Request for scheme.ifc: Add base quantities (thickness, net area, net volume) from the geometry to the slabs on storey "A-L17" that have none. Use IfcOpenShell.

First a look at what the model holds.

```python
import ifcopenshell
import ifcopenshell.util.element
import ifcopenshell.util.unit

model = ifcopenshell.open("scheme.ifc")
print(model.schema)
for unit_type in ("LENGTHUNIT", "AREAUNIT", "VOLUMEUNIT"):
    print(unit_type, ifcopenshell.util.unit.calculate_unit_scale(model, unit_type))
storey = next(s for s in model.by_type("IfcBuildingStorey") if s.Name == "A-L17")
slabs = [e for e in ifcopenshell.util.element.get_decomposition(storey) if e.is_a("IfcSlab")]
for e in sorted(slabs, key=lambda e: e.id()):
    print(e.id(), e.is_a(), e.Name, list(ifcopenshell.util.element.get_psets(e, qtos_only=True)), sep=" | ")
```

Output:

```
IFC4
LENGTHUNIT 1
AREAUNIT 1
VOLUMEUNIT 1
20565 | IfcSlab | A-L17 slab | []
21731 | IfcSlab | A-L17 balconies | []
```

```python
import ifcopenshell
import ifcopenshell.api.pset
import ifcopenshell.geom
import ifcopenshell.util.element
import ifcopenshell.util.shape
import ifcopenshell.util.unit

model = ifcopenshell.open("scheme.ifc")
unit_scale = ifcopenshell.util.unit.calculate_unit_scale(model)
area_scale = ifcopenshell.util.unit.calculate_unit_scale(model, "AREAUNIT")
volume_scale = ifcopenshell.util.unit.calculate_unit_scale(model, "VOLUMEUNIT")
settings = ifcopenshell.geom.settings()

storey = next(s for s in model.by_type("IfcBuildingStorey") if s.Name == "A-L17")
slabs = [e for e in ifcopenshell.util.element.get_decomposition(storey) if e.is_a("IfcSlab")]

for e in sorted(slabs, key=lambda e: e.id()):
    if ifcopenshell.util.element.get_psets(e, qtos_only=True, should_inherit=False):
        continue
    # Geometry comes back in metres, in the element's own axes.
    shape = ifcopenshell.geom.create_shape(settings, e)
    values = {
        "Width": ifcopenshell.util.shape.get_z(shape.geometry) / unit_scale,
        "NetArea": ifcopenshell.util.shape.get_footprint_area(shape.geometry) / area_scale,
        "NetVolume": ifcopenshell.util.shape.get_volume(shape.geometry) / volume_scale,
    }
    qto = ifcopenshell.api.pset.add_qto(model, product=e, name="Qto_SlabBaseQuantities")
    ifcopenshell.api.pset.edit_qto(model, qto=qto, properties=values)
    print(e.id(), {k: round(v, 3) for k, v in values.items()})

model.write("scheme_v2.ifc")
```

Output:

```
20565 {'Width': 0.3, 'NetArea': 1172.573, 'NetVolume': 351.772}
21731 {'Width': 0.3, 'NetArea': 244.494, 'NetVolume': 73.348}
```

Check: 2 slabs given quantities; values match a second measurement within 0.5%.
